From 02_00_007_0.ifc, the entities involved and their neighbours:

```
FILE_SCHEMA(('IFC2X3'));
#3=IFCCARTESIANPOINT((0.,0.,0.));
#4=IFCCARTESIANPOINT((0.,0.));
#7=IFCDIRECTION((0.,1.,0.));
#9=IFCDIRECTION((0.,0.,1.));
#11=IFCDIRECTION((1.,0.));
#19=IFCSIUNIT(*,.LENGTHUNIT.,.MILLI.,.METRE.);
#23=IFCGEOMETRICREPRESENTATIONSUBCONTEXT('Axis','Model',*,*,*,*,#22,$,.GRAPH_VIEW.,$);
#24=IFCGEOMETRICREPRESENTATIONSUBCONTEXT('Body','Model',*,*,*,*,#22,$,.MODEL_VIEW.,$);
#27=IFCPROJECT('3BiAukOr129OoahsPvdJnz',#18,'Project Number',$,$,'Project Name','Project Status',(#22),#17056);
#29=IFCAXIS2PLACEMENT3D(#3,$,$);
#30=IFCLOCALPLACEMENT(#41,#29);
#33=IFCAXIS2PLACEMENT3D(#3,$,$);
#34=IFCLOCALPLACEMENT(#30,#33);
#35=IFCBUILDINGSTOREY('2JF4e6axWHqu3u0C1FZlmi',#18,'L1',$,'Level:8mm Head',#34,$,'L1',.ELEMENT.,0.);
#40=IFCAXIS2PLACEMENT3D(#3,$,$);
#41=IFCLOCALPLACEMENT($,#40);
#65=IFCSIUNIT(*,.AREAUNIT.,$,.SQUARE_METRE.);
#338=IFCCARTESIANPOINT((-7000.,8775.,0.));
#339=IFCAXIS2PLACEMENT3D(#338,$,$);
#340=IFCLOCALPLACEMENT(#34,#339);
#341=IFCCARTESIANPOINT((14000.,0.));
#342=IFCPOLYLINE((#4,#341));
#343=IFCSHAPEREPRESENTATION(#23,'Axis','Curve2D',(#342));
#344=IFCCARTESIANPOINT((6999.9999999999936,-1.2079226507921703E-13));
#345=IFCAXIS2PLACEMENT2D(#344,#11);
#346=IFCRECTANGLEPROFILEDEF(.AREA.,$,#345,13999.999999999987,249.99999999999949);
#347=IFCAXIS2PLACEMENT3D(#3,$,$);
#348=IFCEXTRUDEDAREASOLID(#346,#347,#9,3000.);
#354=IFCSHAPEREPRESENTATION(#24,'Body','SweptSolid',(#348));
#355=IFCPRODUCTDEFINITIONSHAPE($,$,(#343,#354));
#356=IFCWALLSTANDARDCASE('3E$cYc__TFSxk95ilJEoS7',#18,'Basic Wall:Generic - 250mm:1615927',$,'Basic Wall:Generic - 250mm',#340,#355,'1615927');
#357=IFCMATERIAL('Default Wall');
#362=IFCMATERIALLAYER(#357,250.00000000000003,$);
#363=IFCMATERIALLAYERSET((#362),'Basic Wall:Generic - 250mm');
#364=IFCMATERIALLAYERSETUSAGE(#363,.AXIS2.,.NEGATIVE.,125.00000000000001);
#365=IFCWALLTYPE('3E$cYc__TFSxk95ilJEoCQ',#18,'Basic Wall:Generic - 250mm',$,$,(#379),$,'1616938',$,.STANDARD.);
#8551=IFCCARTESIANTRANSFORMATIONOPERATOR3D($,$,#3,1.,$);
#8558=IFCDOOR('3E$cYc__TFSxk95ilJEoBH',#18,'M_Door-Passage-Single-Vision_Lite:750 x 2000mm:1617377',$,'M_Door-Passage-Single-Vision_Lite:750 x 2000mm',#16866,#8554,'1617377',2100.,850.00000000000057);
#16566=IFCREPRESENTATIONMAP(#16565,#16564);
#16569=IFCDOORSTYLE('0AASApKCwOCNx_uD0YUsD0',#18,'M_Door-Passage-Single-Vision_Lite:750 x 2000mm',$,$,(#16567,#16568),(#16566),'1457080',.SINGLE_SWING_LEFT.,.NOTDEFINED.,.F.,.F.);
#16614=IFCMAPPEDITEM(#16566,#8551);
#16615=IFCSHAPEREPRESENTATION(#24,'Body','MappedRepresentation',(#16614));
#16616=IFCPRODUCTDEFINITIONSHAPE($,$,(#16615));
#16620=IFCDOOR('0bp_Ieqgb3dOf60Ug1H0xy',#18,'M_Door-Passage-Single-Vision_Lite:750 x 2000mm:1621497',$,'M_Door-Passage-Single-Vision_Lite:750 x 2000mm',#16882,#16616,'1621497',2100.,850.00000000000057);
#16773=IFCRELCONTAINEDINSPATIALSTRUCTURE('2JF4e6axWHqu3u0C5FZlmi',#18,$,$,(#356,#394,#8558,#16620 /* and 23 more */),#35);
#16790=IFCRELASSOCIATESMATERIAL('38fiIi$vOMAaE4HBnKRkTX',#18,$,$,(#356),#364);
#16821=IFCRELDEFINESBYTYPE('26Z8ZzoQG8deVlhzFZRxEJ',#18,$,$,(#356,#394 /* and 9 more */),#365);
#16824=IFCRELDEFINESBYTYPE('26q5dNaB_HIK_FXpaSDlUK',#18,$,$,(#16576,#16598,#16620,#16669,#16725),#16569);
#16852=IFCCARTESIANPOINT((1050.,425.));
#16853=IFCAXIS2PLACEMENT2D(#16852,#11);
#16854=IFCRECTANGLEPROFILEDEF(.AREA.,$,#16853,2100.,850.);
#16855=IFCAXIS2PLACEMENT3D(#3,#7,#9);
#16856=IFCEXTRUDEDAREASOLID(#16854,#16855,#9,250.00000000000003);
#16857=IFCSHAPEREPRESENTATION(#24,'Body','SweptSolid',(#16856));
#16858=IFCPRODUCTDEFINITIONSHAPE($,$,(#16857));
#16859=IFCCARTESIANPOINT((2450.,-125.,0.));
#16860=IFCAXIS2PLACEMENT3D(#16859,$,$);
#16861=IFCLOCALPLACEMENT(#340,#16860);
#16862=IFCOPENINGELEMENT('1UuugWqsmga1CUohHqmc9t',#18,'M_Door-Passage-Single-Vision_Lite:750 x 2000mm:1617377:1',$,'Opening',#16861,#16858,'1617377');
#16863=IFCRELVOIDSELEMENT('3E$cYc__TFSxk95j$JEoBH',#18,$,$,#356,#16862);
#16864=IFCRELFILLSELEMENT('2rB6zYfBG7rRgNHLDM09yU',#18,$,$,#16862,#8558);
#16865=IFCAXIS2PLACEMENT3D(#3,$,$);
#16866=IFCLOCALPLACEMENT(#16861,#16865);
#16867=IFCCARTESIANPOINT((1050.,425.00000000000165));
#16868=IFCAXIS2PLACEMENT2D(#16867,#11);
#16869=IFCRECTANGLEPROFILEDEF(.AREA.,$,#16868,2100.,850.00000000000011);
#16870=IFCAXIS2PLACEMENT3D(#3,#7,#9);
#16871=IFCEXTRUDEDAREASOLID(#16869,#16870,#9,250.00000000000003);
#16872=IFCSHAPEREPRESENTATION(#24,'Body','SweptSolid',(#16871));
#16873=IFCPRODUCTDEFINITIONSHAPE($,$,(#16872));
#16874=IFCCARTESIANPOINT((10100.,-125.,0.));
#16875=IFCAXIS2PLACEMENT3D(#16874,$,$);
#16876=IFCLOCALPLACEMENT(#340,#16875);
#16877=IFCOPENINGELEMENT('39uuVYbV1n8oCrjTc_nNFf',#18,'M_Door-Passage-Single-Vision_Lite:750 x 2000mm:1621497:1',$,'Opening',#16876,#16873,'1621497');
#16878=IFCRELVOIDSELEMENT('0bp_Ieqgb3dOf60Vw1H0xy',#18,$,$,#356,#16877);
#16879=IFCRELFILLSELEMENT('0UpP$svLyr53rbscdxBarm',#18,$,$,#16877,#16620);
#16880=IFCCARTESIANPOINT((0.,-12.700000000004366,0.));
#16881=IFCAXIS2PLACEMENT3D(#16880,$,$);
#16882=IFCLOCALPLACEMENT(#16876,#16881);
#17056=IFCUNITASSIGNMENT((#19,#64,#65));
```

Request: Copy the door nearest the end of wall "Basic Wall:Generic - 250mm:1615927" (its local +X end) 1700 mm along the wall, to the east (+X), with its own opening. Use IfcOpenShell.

```python
import ifcopenshell
import ifcopenshell.api.feature
import ifcopenshell.api.geometry
import ifcopenshell.api.root
import ifcopenshell.geom
import ifcopenshell.util.element
import ifcopenshell.util.placement
import ifcopenshell.util.shape

model = ifcopenshell.open("02_00_007_0.ifc")
settings = ifcopenshell.geom.settings()


def volume(element):
    """Net volume in cubic metres, openings subtracted."""
    shape = ifcopenshell.geom.create_shape(settings, element)
    return ifcopenshell.util.shape.get_volume(shape.geometry)


def reuse_history(source, copy):
    """copy_class also copies each property set's owner history, people and application; keep the originals."""
    for rel in copy.IsDefinedBy:
        if rel.is_a("IfcRelDefinesByProperties") and (history := rel.RelatingPropertyDefinition.OwnerHistory):
            rel.RelatingPropertyDefinition.OwnerHistory = source.OwnerHistory
            ifcopenshell.util.element.remove_deep2(model, history)


door = model.by_guid("0bp_Ieqgb3dOf60Ug1H0xy")
opening = door.FillsVoids[0].RelatingOpeningElement
wall = opening.VoidsElements[0].RelatingBuildingElement
before = volume(wall)
shift = ifcopenshell.util.placement.get_local_placement(wall.ObjectPlacement)[:3, 0] * 1700.0

# copy_class copies the void relationship, type, container and properties, but no geometry.
new_opening = ifcopenshell.api.root.copy_class(model, product=opening)
new_opening.Representation = ifcopenshell.util.element.copy_deep(
    model, opening.Representation, exclude=["IfcGeometricRepresentationContext", "IfcRepresentationMap"]
)
new_opening.Name = "M_Door-Passage-Single-Vision_Lite:750 x 2000mm"
new_opening.Tag = None
new_door = ifcopenshell.api.root.copy_class(model, product=door)
new_door.Representation = ifcopenshell.util.element.copy_deep(
    model, door.Representation, exclude=["IfcGeometricRepresentationContext", "IfcRepresentationMap"]
)
new_door.Name = "M_Door-Passage-Single-Vision_Lite:750 x 2000mm"
new_door.Tag = None
reuse_history(door, new_door)
fills = ifcopenshell.api.feature.add_filling(model, opening=new_opening, element=new_door)
fills.OwnerHistory = new_door.OwnerHistory  # required in IFC2X3

for old, new in ((opening, new_opening), (door, new_door)):
    matrix = ifcopenshell.util.placement.get_local_placement(old.ObjectPlacement)
    matrix[:3, 3] += shift
    ifcopenshell.api.geometry.edit_object_placement(model, product=new, matrix=matrix, is_si=False)

after = volume(wall)

print(f"wall volume {before:.3f} -> {after:.3f} m3")

model.write("02_00_007_0_v2.ifc")
```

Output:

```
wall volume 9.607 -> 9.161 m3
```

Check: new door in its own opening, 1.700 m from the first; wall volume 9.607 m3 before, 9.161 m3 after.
